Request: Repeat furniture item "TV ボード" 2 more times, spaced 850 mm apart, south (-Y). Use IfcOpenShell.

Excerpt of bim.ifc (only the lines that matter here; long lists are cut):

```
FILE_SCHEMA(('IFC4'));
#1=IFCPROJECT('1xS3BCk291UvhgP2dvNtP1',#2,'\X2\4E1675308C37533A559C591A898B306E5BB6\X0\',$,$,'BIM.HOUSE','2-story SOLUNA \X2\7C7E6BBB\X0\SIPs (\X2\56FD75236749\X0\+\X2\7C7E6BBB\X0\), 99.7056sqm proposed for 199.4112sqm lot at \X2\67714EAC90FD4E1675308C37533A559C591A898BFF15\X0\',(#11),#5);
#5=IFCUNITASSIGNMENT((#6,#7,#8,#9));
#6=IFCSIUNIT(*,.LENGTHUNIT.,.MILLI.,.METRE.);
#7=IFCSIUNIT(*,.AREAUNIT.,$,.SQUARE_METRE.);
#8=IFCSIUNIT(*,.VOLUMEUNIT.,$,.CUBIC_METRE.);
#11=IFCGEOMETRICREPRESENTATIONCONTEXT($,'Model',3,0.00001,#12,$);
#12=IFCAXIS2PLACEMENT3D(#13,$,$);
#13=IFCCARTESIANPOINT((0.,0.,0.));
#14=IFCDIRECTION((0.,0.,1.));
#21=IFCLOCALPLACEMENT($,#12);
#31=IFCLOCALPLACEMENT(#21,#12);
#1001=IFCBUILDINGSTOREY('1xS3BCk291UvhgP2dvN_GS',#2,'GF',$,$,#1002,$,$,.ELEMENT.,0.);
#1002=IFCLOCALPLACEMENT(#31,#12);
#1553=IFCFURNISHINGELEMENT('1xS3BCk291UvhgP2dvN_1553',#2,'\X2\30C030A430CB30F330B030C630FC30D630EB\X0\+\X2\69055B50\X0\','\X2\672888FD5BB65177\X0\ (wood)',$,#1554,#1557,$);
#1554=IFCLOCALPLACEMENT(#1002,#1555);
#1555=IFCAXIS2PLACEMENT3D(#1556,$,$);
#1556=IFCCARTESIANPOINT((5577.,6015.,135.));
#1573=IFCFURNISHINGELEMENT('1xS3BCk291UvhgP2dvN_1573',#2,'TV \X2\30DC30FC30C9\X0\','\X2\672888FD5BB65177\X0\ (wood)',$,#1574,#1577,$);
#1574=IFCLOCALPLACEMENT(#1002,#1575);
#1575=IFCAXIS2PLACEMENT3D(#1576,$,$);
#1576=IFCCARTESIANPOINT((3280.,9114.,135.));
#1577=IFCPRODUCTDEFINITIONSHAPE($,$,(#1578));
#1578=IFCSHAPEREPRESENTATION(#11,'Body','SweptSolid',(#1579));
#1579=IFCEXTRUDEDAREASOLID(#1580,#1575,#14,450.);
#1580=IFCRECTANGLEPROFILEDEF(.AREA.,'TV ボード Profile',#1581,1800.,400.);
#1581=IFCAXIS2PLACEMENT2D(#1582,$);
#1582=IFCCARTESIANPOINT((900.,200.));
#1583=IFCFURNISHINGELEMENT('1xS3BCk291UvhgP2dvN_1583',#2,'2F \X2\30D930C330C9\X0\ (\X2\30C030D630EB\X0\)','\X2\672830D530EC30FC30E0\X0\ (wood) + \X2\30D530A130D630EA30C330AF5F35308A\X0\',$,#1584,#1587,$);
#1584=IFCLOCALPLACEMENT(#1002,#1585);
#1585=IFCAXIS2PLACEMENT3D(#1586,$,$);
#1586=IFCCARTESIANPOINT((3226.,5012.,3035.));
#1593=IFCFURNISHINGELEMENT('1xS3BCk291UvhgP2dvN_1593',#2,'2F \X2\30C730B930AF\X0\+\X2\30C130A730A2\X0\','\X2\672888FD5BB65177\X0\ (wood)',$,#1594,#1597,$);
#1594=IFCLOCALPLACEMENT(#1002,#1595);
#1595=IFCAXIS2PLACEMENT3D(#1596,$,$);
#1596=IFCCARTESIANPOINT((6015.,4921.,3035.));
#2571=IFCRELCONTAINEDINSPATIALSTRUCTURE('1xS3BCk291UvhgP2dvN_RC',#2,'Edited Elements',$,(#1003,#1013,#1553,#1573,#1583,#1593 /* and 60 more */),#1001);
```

```python
import numpy as np
import ifcopenshell
import ifcopenshell.api.geometry
import ifcopenshell.api.root
import ifcopenshell.util.element
import ifcopenshell.util.placement

model = ifcopenshell.open("bim.ifc")


def reuse_history(source, copy):
    """copy_class also copies each property set's owner history, people and application; keep the originals."""
    for rel in copy.IsDefinedBy:
        if rel.is_a("IfcRelDefinesByProperties") and (history := rel.RelatingPropertyDefinition.OwnerHistory):
            rel.RelatingPropertyDefinition.OwnerHistory = source.OwnerHistory
            ifcopenshell.util.element.remove_deep2(model, history)


source = model.by_id(1573)
base = ifcopenshell.util.placement.get_local_placement(source.ObjectPlacement)
step = np.array([0.0, -1.0, 0.0]) * 850.0

for i in range(1, 3):
    copy = ifcopenshell.api.root.copy_class(model, product=source)
    copy.Representation = ifcopenshell.util.element.copy_deep(
        model, source.Representation, exclude=["IfcGeometricRepresentationContext", "IfcRepresentationMap"]
    )
    reuse_history(source, copy)
    matrix = base.copy()
    matrix[:3, 3] += i * step
    print("added at", matrix[:3, 3].round(3) + 0.0)
    ifcopenshell.api.geometry.edit_object_placement(model, product=copy, matrix=matrix, is_si=False)

model.write("bim_edited.ifc")
```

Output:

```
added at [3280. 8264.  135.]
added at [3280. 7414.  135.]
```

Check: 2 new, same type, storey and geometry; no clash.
